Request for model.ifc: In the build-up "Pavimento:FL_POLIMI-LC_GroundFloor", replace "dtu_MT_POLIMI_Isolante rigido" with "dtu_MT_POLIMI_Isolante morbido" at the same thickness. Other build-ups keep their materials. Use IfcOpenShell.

First a look at what the model holds.

```python
import ifcopenshell
import ifcopenshell.util.element

model = ifcopenshell.open("model.ifc")
print(model.schema)
for layer_set in model.by_type("IfcMaterialLayerSet"):
    if layer_set.LayerSetName == "Pavimento:FL_POLIMI-LC_GroundFloor":
        for layer in layer_set.MaterialLayers:
            print(layer.id(), layer.Material and layer.Material.Name, layer.LayerThickness, sep=" | ")
        print(len(ifcopenshell.util.element.get_elements_by_material(model, layer_set)), "elements and types use it")
print(sorted(m.Name for m in model.by_type("IfcMaterial") if m.Name)[:60])
```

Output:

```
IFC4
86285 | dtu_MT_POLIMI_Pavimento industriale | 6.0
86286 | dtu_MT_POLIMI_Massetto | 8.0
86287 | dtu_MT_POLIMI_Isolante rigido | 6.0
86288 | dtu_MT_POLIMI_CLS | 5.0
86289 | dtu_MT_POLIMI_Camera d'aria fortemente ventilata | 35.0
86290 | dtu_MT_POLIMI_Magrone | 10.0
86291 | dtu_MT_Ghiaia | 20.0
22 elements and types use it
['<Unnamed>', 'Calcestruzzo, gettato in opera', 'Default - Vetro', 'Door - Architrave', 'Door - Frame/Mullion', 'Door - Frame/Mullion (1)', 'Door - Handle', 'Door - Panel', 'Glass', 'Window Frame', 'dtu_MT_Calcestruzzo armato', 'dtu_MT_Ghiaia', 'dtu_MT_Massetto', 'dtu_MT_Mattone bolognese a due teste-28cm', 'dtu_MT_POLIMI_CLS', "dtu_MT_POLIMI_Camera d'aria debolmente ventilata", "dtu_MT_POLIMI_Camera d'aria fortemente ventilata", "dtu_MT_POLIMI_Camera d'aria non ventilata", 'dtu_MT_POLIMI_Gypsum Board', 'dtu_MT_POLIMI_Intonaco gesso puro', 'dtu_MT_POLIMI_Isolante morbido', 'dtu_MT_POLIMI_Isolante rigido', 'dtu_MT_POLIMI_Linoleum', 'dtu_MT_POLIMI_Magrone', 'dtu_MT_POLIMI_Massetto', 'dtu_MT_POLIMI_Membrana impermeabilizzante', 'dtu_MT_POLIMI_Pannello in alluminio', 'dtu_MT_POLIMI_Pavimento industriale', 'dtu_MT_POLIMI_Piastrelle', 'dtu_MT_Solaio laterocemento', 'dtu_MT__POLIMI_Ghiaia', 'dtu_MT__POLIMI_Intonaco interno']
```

```python
import ifcopenshell
import ifcopenshell.api.material

model = ifcopenshell.open("model.ifc")

layer_set = next(s for s in model.by_type("IfcMaterialLayerSet") if s.LayerSetName == "Pavimento:FL_POLIMI-LC_GroundFloor")
layer = next(l for l in layer_set.MaterialLayers if l.Material and l.Material.Name == "dtu_MT_POLIMI_Isolante rigido")
material = next(m for m in model.by_type("IfcMaterial") if m.Name == "dtu_MT_POLIMI_Isolante morbido")

# Point this one layer at the other material; renaming the old one would change it everywhere.
ifcopenshell.api.material.edit_layer(model, layer=layer, attributes={"Name": material.Name}, material=material)

print([l.Material.Name if l.Material else None for l in layer_set.MaterialLayers])

model.write("model_updated.ifc")
```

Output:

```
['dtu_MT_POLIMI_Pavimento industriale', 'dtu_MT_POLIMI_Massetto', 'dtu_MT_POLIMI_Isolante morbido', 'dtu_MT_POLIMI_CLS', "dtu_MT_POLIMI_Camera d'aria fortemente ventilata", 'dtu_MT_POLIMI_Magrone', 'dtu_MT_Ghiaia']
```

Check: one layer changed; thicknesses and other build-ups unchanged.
